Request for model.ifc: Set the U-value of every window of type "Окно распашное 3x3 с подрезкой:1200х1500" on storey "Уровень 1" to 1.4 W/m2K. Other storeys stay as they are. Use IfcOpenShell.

First a look at what the model holds.

```python
import ifcopenshell
import ifcopenshell.util.element

model = ifcopenshell.open("model.ifc")
print(model.schema)
storey = next(s for s in model.by_type("IfcBuildingStorey") if s.Name == "Уровень 1")
windows = [e for e in ifcopenshell.util.element.get_decomposition(storey) if e.is_a("IfcWindow")]
seen = {}
for e in windows:
    element_type = ifcopenshell.util.element.get_type(e)
    key = (element_type.Name if element_type != e and element_type else None, ifcopenshell.util.element.get_pset(e, "Pset_WindowCommon", "ThermalTransmittance"))
    seen[key] = seen.get(key, 0) + 1
for (name, value), count in sorted(seen.items(), key=str):
    print(count, "x", name, "|", value)
```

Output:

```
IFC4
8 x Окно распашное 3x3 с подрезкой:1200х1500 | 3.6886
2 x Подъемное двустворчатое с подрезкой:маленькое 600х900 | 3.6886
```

```python
import ifcopenshell
import ifcopenshell.api.pset
import ifcopenshell.util.element

model = ifcopenshell.open("model.ifc")

storey = next(s for s in model.by_type("IfcBuildingStorey") if s.Name == "Уровень 1")
windows = [e for e in ifcopenshell.util.element.get_decomposition(storey) if e.is_a("IfcWindow")]

count = 0
for e in windows:
    element_type = ifcopenshell.util.element.get_type(e)
    if element_type in (None, e) or element_type.Name != "Окно распашное 3x3 с подрезкой:1200х1500":
        continue
    # add_pset returns the element's existing set when there is one.
    pset = ifcopenshell.api.pset.add_pset(model, product=e, name="Pset_WindowCommon")
    ifcopenshell.api.pset.edit_pset(model, pset=pset, properties={"ThermalTransmittance": 1.4})
    count += 1

print(count, "windows updated")

model.write("model_rev.ifc")
```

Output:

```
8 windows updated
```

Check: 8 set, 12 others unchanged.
